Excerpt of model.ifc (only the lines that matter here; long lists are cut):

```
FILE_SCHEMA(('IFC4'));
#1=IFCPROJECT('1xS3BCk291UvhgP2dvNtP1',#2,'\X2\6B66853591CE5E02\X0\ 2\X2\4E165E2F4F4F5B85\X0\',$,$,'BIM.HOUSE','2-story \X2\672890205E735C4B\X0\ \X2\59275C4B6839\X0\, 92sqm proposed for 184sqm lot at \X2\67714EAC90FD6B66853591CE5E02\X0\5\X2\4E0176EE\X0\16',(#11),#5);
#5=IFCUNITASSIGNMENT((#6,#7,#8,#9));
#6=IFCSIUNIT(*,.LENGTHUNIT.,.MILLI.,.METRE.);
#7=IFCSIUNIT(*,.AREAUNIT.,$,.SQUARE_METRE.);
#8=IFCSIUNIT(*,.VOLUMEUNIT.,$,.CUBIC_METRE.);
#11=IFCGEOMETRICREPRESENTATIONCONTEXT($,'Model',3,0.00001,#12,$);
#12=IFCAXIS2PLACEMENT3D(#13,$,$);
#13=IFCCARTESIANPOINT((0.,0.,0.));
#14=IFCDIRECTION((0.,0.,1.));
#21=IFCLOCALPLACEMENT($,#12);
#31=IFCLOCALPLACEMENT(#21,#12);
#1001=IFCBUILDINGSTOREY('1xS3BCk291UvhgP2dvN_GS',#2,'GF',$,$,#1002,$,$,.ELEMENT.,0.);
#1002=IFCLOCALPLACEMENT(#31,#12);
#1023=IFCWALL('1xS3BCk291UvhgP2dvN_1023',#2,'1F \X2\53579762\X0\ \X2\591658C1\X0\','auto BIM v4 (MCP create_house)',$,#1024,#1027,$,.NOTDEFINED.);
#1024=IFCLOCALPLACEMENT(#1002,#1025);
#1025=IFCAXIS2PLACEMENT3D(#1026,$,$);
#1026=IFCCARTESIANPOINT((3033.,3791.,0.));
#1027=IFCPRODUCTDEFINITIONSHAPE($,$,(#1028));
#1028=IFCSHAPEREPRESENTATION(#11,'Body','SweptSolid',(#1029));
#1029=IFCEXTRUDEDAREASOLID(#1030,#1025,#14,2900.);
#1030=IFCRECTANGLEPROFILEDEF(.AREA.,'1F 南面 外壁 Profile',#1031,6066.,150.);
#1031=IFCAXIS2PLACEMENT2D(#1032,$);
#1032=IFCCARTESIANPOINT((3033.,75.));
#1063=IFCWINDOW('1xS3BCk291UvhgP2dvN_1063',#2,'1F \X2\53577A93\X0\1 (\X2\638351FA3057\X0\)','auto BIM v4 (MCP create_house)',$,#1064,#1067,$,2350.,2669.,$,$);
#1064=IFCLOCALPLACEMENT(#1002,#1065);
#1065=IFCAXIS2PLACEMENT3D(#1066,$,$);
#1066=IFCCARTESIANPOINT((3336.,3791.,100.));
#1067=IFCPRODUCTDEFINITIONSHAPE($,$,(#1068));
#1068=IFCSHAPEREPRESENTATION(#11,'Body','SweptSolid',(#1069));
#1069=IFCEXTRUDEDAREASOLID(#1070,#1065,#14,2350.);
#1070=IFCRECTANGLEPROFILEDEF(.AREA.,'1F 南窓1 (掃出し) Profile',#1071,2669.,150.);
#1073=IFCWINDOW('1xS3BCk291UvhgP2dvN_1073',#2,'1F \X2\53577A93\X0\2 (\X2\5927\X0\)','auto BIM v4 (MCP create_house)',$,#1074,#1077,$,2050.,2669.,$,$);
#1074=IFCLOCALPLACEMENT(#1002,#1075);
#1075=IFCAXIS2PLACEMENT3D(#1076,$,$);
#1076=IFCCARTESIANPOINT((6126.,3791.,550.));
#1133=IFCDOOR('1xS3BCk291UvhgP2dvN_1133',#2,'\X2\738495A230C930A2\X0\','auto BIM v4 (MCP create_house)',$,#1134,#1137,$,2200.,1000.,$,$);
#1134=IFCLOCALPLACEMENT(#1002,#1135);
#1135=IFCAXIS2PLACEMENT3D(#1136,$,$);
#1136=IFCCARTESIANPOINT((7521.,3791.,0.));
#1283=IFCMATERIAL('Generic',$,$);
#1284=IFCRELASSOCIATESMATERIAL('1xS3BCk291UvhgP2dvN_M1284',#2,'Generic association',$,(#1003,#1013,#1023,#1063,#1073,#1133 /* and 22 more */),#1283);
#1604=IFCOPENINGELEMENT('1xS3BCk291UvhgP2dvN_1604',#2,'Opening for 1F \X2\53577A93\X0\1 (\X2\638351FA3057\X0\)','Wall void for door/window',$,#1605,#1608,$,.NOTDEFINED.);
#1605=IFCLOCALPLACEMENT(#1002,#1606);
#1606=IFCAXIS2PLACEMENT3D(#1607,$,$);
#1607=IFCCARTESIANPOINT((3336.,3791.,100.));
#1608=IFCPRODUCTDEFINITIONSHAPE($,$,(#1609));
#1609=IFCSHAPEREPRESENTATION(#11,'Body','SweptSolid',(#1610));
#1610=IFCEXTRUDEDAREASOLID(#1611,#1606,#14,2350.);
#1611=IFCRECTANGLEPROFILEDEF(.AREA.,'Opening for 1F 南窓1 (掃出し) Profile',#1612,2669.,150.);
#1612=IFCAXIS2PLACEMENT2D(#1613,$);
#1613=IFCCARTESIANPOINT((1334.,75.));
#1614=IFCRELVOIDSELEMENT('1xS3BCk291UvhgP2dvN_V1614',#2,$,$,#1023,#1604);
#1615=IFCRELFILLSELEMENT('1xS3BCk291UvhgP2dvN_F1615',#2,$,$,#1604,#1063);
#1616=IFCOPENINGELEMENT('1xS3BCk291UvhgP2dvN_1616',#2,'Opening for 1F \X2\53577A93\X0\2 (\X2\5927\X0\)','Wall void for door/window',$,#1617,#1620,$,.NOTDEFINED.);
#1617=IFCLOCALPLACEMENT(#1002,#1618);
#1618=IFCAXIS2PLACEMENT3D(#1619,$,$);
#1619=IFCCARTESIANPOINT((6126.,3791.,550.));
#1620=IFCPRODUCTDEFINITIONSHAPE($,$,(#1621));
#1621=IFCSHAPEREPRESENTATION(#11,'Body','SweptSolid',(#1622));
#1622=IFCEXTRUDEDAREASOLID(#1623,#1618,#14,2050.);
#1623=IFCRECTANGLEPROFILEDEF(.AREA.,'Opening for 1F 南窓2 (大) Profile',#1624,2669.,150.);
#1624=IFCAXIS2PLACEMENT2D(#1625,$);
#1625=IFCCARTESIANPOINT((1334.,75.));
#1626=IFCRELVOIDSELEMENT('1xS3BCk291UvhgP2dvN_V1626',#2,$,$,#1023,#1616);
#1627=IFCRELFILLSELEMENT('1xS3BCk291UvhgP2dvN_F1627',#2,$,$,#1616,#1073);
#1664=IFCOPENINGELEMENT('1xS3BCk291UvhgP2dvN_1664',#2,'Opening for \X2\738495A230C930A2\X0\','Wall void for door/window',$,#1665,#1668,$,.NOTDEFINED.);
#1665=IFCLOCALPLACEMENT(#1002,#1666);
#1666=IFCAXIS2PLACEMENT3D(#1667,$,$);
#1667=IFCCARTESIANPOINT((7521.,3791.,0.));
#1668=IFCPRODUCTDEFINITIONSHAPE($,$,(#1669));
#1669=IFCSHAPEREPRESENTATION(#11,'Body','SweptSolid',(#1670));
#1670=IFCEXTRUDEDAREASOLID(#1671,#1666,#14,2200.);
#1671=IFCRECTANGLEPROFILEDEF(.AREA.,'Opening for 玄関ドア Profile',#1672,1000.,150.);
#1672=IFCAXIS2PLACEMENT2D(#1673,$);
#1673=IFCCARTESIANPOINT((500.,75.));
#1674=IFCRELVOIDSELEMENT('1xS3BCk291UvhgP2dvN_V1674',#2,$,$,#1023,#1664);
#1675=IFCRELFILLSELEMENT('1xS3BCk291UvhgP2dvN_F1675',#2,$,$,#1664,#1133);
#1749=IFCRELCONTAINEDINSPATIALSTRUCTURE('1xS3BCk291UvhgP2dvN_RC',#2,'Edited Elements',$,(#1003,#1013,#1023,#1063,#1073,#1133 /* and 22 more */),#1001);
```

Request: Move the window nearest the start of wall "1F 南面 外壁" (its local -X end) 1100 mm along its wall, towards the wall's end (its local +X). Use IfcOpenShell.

```python
import ifcopenshell
import ifcopenshell.api.geometry
import ifcopenshell.util.placement
import ifcopenshell.util.unit

model = ifcopenshell.open("model.ifc")
unit_scale = ifcopenshell.util.unit.calculate_unit_scale(model)

window = model.by_guid("1xS3BCk291UvhgP2dvN_1063")
opening = window.FillsVoids[0].RelatingOpeningElement
wall = opening.VoidsElements[0].RelatingBuildingElement

wall_matrix = ifcopenshell.util.placement.get_local_placement(wall.ObjectPlacement)
shift = wall_matrix[:3, 0] * 1.1 / unit_scale
before = ifcopenshell.util.placement.get_local_placement(window.ObjectPlacement)[:3, 3].copy()

# The window is not placed relative to its opening, so move both.
for product in (opening, window):
    matrix = ifcopenshell.util.placement.get_local_placement(product.ObjectPlacement)
    matrix[:3, 3] += shift
    ifcopenshell.api.geometry.edit_object_placement(model, product=product, matrix=matrix, is_si=False)

after = ifcopenshell.util.placement.get_local_placement(window.ObjectPlacement)[:3, 3]
print("window moved by", (after - before).round(3) + 0.0)

model.write("model_edited.ifc")
```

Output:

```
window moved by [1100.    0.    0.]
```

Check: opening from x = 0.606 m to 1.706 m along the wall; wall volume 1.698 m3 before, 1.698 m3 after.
